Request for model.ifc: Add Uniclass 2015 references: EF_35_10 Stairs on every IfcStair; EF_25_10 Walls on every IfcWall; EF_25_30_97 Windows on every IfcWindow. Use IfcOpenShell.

First a look at what the model holds.

```python
import ifcopenshell

model = ifcopenshell.open("model.ifc")
print(model.schema)
print("classifications:", [c.Name for c in model.by_type("IfcClassification")])
for ifc_class in ("IfcDoor", "IfcRoof", "IfcStair", "IfcWall", "IfcWindow"):
    print(ifc_class, len(model.by_type(ifc_class)))
```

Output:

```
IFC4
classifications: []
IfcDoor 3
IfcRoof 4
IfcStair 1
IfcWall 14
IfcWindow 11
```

```python
import ifcopenshell
import ifcopenshell.api.classification

model = ifcopenshell.open("model.ifc")

system = ifcopenshell.api.classification.add_classification(model, classification="Uniclass 2015")

codes = {
    "IfcStair": ("EF_35_10", "Stairs"),
    "IfcWall": ("EF_25_10", "Walls"),
    "IfcWindow": ("EF_25_30_97", "Windows"),
}
for ifc_class, (code, name) in codes.items():
    products = model.by_type(ifc_class)
    ifcopenshell.api.classification.add_reference(
        model, products=products, classification=system, identification=code, name=name
    )
    print(code, len(products))

model.write("model-out.ifc")
```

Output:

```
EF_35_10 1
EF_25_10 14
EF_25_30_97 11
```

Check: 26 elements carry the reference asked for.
